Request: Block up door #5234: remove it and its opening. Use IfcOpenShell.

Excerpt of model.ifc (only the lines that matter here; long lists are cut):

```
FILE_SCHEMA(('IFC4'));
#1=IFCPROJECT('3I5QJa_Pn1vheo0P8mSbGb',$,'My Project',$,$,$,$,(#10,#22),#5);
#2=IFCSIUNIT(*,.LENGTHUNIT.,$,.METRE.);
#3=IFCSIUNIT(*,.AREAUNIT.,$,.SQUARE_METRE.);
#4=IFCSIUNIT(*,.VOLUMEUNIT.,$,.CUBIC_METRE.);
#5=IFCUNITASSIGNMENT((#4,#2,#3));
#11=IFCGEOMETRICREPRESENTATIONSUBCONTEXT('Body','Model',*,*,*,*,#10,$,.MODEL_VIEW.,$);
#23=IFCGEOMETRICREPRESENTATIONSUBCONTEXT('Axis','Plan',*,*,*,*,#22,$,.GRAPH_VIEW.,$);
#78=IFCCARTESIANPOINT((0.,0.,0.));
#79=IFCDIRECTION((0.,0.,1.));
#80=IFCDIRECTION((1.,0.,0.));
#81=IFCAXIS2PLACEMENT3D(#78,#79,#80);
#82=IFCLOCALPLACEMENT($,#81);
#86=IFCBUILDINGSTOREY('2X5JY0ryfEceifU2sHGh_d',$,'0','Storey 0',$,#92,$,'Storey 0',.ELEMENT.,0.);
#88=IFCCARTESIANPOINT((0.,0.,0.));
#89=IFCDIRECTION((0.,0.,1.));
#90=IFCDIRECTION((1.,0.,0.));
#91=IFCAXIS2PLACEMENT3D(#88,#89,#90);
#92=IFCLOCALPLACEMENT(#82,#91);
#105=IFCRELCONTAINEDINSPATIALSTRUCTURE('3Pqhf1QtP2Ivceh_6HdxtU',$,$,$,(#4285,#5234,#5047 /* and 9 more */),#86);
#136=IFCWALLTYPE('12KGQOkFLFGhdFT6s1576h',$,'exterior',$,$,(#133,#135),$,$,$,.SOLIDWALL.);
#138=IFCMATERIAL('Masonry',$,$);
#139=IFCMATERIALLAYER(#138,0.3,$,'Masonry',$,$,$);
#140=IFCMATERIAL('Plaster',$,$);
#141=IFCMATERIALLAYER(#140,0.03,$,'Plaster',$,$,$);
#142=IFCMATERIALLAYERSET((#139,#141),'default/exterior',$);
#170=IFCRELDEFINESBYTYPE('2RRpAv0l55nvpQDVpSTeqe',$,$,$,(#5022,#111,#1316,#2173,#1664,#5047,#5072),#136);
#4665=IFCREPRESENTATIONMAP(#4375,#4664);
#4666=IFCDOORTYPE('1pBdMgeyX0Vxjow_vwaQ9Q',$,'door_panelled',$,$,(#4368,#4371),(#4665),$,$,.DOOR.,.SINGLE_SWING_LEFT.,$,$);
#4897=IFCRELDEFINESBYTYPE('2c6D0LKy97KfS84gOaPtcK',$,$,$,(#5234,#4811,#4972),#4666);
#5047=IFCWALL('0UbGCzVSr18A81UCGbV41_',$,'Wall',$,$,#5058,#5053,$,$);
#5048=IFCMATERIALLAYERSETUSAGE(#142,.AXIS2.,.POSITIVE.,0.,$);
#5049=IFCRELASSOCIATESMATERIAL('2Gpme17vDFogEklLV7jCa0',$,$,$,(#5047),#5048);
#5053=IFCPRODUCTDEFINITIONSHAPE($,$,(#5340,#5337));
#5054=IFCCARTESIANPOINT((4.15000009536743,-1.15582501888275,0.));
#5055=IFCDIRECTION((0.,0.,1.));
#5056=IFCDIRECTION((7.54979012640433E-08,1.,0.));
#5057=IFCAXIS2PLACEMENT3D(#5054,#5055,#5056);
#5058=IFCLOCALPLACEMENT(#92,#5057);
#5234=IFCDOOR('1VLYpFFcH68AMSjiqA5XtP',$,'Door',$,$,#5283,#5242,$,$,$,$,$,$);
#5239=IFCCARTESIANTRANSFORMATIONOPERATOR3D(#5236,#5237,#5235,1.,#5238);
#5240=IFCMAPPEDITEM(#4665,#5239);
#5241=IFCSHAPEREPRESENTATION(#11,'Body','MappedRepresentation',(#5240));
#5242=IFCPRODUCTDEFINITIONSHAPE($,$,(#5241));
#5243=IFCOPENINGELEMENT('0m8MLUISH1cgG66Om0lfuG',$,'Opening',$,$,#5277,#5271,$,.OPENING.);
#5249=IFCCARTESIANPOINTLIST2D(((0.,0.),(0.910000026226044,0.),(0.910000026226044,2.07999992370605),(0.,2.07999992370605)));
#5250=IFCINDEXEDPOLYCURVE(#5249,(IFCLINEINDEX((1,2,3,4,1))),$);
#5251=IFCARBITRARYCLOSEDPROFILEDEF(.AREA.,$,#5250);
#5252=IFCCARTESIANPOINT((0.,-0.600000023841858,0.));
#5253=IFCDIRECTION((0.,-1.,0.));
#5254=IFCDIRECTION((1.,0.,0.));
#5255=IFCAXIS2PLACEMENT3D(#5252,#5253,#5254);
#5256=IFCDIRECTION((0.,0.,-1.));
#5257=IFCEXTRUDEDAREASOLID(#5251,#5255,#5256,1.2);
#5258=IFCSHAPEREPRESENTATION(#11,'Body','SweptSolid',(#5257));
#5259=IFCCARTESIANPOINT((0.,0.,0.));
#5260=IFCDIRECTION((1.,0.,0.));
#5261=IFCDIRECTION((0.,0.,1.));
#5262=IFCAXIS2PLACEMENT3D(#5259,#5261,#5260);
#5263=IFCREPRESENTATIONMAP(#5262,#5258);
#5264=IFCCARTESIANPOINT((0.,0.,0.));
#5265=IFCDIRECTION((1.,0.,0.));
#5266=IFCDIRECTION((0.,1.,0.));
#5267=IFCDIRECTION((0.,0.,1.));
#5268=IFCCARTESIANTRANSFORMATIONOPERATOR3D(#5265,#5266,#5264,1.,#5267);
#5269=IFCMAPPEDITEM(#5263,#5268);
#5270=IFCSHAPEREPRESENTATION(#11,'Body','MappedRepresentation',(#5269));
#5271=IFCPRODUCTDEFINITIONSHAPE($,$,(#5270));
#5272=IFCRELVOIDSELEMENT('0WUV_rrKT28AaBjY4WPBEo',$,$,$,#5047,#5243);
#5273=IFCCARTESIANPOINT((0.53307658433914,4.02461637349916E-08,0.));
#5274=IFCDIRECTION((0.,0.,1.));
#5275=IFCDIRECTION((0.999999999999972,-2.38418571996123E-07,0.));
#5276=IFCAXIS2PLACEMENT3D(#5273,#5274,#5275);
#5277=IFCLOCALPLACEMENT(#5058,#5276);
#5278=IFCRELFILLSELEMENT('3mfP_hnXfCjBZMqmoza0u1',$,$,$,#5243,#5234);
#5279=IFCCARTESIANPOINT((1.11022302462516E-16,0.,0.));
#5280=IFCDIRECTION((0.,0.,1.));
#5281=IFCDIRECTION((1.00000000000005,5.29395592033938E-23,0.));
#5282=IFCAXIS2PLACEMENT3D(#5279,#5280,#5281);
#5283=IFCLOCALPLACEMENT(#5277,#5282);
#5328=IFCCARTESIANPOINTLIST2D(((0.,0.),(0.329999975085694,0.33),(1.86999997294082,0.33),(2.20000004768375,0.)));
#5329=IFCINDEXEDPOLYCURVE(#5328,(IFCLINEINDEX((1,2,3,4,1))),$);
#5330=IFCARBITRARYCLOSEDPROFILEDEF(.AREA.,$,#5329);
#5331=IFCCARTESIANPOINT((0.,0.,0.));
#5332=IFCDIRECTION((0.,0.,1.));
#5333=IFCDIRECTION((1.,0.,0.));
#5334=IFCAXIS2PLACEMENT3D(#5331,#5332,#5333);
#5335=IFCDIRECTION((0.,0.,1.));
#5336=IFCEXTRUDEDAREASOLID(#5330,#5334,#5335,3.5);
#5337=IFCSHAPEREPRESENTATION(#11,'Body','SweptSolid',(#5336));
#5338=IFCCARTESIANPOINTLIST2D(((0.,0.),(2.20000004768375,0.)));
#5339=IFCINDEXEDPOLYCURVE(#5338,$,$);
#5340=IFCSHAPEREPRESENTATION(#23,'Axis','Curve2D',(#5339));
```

```python
import ifcopenshell
import ifcopenshell.api.feature
import ifcopenshell.api.root
import ifcopenshell.geom
import ifcopenshell.util.shape

model = ifcopenshell.open("model.ifc")
settings = ifcopenshell.geom.settings()


def volume(element):
    """Net volume in cubic metres, openings subtracted."""
    shape = ifcopenshell.geom.create_shape(settings, element)
    return ifcopenshell.util.shape.get_volume(shape.geometry)


door = model.by_id(5234)
opening = door.FillsVoids[0].RelatingOpeningElement
wall = opening.VoidsElements[0].RelatingBuildingElement
before = volume(wall)

ifcopenshell.api.root.remove_product(model, product=door)
ifcopenshell.api.feature.remove_feature(model, feature=opening)

after = volume(wall)

print(f"wall volume {before:.3f} -> {after:.3f} m3")

model.write("model-out.ifc")
```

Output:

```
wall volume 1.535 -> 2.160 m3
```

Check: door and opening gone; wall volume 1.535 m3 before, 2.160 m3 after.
